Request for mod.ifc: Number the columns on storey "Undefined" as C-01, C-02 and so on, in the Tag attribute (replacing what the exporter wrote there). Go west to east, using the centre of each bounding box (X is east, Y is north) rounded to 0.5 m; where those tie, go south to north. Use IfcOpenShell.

First a look at what the model holds.

```python
import ifcopenshell
import ifcopenshell.util.element
import ifcopenshell.util.placement

model = ifcopenshell.open("mod.ifc")
print(model.schema)
storey = next(s for s in model.by_type("IfcBuildingStorey") if s.Name == "Undefined")
columns = [e for e in ifcopenshell.util.element.get_decomposition(storey) if e.is_a("IfcColumn")]
for e in sorted(columns, key=lambda e: e.id()):
    origin = ifcopenshell.util.placement.get_local_placement(e.ObjectPlacement)[:3, 3]
    print(e.id(), e.Tag, e.Name, origin.round(2) + 0.0, sep=" | ")
```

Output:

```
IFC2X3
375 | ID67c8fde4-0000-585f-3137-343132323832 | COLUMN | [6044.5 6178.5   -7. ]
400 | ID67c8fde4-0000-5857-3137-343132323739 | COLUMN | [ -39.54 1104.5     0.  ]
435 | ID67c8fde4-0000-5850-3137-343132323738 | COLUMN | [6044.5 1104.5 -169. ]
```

```python
import ifcopenshell
import ifcopenshell.geom
import ifcopenshell.util.element
import ifcopenshell.util.shape

model = ifcopenshell.open("mod.ifc")
settings = ifcopenshell.geom.settings()
settings.set("use-world-coords", True)


def centre(element):
    shape = ifcopenshell.geom.create_shape(settings, element)
    return ifcopenshell.util.shape.get_bbox_centroid(shape.geometry)


storey = next(s for s in model.by_type("IfcBuildingStorey") if s.Name == "Undefined")
columns = [e for e in ifcopenshell.util.element.get_decomposition(storey) if e.is_a("IfcColumn")]

# Insertion points can sit at a corner or the storey origin, so sort by the geometry (in metres).
centres = {e: centre(e) for e in columns}
columns.sort(key=lambda e: (round(centres[e][0] / 0.5), centres[e][1]))

for i, e in enumerate(columns, start=1):
    number = f"C-{i:02d}"
    e.Tag = number
    print(e.id(), number)

model.write("mod_rev.ifc")
```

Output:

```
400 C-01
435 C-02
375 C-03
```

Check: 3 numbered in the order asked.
